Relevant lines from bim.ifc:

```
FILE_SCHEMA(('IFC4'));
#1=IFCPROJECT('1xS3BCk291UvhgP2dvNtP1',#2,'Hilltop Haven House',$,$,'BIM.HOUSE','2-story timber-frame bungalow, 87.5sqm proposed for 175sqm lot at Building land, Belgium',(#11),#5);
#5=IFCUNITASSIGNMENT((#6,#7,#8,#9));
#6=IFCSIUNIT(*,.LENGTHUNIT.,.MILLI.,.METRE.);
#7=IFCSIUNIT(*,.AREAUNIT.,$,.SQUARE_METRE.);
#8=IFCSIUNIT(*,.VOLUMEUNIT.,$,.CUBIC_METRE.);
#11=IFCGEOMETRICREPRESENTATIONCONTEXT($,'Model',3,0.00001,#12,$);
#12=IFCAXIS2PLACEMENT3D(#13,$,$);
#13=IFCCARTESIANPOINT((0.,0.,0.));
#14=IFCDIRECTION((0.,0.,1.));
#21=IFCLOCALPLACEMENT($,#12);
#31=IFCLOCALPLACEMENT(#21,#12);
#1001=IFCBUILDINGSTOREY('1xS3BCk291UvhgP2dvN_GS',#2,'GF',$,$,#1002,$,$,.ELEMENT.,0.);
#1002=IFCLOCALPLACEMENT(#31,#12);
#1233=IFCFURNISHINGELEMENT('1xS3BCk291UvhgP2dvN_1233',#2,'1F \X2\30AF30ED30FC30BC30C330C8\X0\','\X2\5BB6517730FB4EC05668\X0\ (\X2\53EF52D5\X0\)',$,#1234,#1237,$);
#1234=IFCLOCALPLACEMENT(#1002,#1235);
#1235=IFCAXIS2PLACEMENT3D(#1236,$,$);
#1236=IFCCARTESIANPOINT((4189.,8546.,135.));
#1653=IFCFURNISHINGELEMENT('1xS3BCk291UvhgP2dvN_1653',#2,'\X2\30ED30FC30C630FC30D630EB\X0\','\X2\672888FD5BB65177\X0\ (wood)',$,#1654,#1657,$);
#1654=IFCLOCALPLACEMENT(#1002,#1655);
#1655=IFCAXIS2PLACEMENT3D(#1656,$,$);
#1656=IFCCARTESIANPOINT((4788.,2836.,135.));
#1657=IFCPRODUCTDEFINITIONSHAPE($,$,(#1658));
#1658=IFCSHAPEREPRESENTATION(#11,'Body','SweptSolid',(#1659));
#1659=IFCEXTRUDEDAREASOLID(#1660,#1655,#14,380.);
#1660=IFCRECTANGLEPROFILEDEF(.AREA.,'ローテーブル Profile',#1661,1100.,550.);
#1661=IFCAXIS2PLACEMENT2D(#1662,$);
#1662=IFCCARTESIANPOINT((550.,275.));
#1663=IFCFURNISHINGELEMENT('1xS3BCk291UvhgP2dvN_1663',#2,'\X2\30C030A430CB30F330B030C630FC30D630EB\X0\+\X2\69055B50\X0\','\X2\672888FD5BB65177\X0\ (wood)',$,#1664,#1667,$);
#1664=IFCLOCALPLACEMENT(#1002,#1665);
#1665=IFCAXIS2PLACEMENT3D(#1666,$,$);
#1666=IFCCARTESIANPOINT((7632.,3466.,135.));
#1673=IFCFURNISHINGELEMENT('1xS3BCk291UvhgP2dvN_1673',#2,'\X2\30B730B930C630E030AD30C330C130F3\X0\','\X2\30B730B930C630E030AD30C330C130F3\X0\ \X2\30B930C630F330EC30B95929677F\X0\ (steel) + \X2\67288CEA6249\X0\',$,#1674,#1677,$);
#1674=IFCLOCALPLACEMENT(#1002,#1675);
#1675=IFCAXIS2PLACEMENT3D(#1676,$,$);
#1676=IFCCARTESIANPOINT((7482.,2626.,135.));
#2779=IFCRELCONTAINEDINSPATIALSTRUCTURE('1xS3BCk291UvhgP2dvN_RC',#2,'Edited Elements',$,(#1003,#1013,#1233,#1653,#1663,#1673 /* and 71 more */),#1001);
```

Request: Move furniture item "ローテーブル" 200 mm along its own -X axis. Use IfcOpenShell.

```python
import ifcopenshell
import ifcopenshell.api.geometry
import ifcopenshell.util.placement
import ifcopenshell.util.unit

model = ifcopenshell.open("bim.ifc")
unit_scale = ifcopenshell.util.unit.calculate_unit_scale(model)

item = model.by_guid("1xS3BCk291UvhgP2dvN_1653")
matrix = ifcopenshell.util.placement.get_local_placement(item.ObjectPlacement)
matrix[:3, 3] -= matrix[:3, 0] * 0.2 / unit_scale
ifcopenshell.api.geometry.edit_object_placement(model, product=item, matrix=matrix, is_si=False)

print(ifcopenshell.util.placement.get_local_placement(item.ObjectPlacement).round(3) + 0.0)

model.write("bim_edited.ifc")
```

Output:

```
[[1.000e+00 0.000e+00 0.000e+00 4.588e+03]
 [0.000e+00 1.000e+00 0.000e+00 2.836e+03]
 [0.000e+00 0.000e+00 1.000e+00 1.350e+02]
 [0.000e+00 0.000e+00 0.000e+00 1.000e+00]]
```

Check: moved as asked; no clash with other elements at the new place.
